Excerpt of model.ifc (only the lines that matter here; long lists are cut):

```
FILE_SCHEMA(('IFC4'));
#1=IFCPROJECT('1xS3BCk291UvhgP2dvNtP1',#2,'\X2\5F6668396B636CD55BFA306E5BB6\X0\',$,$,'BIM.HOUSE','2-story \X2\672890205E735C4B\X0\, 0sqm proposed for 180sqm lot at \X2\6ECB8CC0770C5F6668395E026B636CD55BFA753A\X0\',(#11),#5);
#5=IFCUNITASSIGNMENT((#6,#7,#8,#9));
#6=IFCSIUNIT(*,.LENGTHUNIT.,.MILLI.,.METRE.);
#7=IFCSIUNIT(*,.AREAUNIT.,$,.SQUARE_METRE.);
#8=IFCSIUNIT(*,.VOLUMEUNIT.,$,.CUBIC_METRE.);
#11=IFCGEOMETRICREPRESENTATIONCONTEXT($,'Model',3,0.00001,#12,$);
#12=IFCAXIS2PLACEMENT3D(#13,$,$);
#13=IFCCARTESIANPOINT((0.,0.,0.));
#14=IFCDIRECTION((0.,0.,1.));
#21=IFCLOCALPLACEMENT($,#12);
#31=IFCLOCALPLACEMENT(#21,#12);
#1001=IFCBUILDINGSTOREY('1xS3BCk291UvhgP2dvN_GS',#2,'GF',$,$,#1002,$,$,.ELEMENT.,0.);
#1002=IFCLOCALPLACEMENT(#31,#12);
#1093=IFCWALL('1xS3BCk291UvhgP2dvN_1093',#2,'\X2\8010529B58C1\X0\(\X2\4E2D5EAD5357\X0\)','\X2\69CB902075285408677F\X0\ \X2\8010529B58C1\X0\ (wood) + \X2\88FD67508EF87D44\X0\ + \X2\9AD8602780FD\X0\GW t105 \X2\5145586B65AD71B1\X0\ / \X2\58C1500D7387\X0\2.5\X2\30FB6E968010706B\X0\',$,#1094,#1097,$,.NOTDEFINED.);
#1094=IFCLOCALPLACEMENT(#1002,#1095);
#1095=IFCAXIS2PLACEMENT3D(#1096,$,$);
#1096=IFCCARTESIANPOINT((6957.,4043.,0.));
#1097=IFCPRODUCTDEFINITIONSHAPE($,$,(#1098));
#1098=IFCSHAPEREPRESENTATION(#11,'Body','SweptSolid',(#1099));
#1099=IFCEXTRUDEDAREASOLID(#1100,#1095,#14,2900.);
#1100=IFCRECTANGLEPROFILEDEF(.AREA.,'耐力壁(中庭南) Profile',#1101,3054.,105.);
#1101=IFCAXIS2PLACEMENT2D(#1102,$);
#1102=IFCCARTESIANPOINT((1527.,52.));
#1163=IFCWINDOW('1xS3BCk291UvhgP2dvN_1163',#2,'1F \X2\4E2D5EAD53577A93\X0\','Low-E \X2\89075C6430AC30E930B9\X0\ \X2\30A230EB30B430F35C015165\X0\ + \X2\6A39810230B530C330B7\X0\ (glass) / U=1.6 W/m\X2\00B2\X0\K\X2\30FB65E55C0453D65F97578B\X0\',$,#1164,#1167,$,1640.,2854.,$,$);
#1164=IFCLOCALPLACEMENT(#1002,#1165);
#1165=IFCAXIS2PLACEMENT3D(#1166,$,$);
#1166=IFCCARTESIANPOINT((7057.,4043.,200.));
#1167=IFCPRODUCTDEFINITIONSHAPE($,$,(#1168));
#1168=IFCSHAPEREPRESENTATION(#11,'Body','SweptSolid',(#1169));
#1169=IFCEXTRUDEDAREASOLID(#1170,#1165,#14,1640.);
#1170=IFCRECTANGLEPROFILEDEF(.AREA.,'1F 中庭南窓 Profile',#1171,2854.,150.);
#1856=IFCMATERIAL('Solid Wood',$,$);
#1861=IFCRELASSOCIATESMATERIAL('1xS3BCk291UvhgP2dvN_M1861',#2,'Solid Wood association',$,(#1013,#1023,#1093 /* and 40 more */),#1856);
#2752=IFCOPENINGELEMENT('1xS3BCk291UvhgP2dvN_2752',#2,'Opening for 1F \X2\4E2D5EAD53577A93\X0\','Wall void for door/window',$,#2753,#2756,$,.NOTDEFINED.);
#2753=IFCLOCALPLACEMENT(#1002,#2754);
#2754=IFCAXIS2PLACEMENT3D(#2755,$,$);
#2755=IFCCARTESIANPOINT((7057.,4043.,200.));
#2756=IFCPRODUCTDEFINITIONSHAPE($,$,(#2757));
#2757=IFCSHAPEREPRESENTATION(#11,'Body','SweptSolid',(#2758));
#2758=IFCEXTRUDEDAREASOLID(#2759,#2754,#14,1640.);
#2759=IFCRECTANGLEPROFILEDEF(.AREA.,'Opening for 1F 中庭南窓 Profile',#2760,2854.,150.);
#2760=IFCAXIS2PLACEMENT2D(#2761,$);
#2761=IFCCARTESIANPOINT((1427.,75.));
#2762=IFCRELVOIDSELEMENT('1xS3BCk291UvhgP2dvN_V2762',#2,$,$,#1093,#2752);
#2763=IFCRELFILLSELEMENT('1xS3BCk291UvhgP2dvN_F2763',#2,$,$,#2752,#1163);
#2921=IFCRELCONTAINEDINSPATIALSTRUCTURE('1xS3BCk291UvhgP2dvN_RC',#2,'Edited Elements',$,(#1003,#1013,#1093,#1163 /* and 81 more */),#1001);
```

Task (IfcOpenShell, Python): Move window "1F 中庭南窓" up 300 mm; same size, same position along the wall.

```python
import numpy as np
import ifcopenshell
import ifcopenshell.api.geometry
import ifcopenshell.util.placement
import ifcopenshell.util.unit

model = ifcopenshell.open("model.ifc")
unit_scale = ifcopenshell.util.unit.calculate_unit_scale(model)

window = model.by_guid("1xS3BCk291UvhgP2dvN_1163")
opening = window.FillsVoids[0].RelatingOpeningElement
dz = 0.3 / unit_scale

shift = np.array([0.0, 0.0, dz])
# The window is not placed relative to its opening, so move both.
for product in (opening, window):
    matrix = ifcopenshell.util.placement.get_local_placement(product.ObjectPlacement)
    matrix[:3, 3] += shift
    ifcopenshell.api.geometry.edit_object_placement(model, product=product, matrix=matrix, is_si=False)

print(f"moved by {dz * unit_scale:+.3f} m")

model.write("model_v2.ifc")
```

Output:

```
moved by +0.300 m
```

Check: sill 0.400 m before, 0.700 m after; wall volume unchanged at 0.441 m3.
